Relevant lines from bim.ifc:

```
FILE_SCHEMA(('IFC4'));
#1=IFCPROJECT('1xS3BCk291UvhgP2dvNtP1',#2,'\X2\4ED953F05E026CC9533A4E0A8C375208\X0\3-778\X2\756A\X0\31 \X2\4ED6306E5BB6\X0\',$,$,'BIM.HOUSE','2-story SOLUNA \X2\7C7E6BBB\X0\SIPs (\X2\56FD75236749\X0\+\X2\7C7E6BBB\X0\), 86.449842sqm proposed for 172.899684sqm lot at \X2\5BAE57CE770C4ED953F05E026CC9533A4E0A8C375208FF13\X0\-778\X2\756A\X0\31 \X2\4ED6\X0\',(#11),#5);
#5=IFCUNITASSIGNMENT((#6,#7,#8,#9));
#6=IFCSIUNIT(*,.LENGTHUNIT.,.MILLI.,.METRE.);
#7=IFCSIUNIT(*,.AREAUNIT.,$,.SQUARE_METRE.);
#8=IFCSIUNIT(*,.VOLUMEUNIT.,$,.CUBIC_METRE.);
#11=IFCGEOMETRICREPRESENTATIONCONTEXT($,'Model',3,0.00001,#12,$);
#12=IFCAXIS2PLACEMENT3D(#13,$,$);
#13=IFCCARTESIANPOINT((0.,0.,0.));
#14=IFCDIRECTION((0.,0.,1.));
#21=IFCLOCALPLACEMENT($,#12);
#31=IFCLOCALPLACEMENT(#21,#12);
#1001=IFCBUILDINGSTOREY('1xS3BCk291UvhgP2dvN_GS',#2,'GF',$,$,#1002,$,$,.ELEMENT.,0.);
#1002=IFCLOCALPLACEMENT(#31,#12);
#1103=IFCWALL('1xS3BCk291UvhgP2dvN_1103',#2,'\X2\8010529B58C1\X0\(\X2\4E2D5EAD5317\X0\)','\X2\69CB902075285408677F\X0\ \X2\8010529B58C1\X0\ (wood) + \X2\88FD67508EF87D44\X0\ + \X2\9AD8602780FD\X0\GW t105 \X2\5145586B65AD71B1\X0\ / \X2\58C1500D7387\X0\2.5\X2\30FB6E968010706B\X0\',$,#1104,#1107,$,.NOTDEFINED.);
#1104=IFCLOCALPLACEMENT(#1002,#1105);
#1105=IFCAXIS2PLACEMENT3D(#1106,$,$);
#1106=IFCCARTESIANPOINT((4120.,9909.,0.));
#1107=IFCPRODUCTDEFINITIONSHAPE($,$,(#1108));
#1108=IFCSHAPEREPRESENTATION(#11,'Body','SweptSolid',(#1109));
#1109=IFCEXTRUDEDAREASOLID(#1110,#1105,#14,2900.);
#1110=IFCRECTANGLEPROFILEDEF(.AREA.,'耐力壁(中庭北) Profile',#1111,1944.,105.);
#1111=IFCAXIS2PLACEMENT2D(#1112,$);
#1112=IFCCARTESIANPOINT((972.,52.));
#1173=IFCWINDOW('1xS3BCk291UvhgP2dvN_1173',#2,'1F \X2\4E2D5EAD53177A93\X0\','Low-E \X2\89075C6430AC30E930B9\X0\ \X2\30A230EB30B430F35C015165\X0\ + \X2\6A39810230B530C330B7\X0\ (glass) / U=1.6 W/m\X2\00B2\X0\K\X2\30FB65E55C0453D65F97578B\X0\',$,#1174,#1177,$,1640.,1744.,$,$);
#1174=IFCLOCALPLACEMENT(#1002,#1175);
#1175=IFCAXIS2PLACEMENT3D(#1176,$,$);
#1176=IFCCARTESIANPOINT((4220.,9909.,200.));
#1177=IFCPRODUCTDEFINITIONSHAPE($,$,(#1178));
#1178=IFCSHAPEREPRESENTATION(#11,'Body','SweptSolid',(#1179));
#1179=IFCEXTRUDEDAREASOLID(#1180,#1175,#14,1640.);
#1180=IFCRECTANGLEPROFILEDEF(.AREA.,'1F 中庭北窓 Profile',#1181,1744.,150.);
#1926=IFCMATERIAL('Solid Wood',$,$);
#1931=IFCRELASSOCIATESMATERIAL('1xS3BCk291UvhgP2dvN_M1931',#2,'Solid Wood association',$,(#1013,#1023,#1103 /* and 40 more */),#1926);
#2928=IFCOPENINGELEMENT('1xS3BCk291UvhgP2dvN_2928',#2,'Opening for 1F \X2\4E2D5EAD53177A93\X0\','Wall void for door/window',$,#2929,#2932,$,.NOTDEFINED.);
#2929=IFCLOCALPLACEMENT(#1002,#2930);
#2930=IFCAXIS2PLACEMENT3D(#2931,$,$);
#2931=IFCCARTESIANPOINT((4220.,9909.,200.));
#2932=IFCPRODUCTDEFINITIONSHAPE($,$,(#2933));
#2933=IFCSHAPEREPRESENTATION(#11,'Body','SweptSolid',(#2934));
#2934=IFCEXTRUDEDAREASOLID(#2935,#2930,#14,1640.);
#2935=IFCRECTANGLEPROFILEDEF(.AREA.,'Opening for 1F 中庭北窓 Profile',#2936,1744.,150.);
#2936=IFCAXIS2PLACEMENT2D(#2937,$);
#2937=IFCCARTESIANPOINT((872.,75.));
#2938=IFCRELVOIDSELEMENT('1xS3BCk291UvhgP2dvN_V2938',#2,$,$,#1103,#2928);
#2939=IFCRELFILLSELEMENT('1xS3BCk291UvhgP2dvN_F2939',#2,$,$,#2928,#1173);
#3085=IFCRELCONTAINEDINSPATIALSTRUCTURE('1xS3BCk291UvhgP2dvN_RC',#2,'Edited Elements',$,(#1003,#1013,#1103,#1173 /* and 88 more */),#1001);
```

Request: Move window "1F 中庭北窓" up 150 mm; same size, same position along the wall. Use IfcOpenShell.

```python
import numpy as np
import ifcopenshell
import ifcopenshell.api.geometry
import ifcopenshell.util.placement
import ifcopenshell.util.unit

model = ifcopenshell.open("bim.ifc")
unit_scale = ifcopenshell.util.unit.calculate_unit_scale(model)

window = model.by_guid("1xS3BCk291UvhgP2dvN_1173")
opening = window.FillsVoids[0].RelatingOpeningElement
dz = 0.15 / unit_scale

shift = np.array([0.0, 0.0, dz])
# The window is not placed relative to its opening, so move both.
for product in (opening, window):
    matrix = ifcopenshell.util.placement.get_local_placement(product.ObjectPlacement)
    matrix[:3, 3] += shift
    ifcopenshell.api.geometry.edit_object_placement(model, product=product, matrix=matrix, is_si=False)

print(f"moved by {dz * unit_scale:+.3f} m")

model.write("bim_v2.ifc")
```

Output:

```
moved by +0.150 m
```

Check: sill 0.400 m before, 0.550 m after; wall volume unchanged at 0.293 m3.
